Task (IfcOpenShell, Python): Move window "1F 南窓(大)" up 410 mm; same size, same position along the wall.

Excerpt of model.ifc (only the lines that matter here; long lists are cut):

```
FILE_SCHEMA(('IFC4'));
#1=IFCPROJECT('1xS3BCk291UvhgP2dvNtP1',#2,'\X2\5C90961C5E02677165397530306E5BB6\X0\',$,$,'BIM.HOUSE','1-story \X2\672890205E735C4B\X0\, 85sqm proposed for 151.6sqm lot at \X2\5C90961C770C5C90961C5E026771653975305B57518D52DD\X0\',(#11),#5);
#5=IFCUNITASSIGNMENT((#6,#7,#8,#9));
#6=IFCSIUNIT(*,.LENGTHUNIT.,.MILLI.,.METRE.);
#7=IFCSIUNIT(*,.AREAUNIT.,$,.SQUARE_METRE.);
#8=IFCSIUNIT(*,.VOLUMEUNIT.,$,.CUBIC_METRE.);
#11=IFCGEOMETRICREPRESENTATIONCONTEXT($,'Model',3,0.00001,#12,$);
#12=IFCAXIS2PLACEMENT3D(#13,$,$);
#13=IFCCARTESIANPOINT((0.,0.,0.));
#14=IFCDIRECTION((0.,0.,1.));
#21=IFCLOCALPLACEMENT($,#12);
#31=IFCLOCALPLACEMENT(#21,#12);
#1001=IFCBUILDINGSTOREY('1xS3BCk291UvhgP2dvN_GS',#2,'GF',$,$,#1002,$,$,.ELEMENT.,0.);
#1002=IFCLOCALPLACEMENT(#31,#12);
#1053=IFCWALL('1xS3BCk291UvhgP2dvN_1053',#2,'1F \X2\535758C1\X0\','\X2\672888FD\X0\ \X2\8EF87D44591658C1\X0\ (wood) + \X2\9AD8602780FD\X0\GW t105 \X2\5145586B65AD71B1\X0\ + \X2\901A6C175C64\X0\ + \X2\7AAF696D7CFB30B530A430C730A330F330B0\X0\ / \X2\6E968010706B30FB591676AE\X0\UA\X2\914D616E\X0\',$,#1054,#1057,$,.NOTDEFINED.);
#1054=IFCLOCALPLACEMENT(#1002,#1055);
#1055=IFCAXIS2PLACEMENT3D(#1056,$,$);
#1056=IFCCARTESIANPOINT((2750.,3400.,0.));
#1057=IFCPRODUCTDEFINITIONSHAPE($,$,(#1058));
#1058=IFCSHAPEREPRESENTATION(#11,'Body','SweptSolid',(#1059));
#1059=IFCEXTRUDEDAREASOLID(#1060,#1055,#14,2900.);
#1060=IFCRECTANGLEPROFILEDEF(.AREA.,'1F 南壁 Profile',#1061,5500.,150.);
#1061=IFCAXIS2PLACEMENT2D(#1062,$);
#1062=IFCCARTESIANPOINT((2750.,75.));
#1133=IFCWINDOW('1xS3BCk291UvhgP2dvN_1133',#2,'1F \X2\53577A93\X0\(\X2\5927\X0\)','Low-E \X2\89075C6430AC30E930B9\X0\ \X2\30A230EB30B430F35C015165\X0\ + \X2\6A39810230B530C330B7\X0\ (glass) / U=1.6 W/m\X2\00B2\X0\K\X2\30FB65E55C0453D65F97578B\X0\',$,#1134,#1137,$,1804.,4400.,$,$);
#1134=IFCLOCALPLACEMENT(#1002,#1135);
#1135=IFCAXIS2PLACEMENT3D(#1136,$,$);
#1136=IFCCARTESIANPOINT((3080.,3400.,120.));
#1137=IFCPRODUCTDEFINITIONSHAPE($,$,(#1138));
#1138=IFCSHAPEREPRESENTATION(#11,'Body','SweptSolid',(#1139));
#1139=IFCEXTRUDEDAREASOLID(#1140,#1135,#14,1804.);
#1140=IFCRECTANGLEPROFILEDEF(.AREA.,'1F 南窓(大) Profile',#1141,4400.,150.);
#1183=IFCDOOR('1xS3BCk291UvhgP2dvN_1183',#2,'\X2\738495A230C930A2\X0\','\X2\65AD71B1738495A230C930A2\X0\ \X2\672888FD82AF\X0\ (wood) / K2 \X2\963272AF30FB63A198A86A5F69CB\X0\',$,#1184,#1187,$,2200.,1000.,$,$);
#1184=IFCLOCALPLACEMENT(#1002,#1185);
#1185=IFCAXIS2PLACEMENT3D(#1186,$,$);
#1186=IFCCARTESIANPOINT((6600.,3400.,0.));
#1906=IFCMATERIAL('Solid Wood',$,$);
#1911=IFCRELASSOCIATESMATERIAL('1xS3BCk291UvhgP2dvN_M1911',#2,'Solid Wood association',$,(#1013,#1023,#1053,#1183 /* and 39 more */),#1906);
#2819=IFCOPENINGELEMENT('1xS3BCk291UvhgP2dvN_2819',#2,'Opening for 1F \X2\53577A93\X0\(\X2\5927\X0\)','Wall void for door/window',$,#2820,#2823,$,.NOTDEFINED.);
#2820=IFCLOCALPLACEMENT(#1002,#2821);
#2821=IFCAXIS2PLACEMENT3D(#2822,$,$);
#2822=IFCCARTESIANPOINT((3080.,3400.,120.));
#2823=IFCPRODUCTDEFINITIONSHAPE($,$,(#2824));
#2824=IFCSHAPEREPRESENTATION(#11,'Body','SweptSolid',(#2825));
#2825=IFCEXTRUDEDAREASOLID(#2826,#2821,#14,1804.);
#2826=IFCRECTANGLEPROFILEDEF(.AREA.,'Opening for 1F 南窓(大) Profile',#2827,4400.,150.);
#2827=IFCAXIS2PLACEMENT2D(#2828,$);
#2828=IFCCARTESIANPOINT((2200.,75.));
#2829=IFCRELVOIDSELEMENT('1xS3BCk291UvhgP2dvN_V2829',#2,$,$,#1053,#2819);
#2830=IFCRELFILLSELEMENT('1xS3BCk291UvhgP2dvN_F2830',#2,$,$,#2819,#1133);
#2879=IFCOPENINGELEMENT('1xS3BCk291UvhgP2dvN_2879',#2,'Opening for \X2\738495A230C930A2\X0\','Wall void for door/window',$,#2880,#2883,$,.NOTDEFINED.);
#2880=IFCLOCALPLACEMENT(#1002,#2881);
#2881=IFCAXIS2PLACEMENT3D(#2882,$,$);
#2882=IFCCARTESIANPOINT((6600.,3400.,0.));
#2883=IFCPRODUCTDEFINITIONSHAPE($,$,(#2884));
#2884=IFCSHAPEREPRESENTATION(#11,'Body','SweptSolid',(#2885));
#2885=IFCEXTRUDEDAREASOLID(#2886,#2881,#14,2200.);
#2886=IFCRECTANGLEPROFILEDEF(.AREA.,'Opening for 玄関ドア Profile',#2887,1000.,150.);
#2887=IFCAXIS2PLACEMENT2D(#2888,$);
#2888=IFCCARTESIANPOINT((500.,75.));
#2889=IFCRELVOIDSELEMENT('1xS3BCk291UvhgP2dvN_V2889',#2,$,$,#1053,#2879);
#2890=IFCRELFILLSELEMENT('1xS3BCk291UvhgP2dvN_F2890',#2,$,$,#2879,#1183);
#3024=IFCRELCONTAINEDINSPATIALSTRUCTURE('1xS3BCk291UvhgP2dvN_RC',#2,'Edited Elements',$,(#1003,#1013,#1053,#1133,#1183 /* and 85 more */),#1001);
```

```python
import numpy as np
import ifcopenshell
import ifcopenshell.api.geometry
import ifcopenshell.util.placement
import ifcopenshell.util.unit

model = ifcopenshell.open("model.ifc")
unit_scale = ifcopenshell.util.unit.calculate_unit_scale(model)

window = model.by_guid("1xS3BCk291UvhgP2dvN_1133")
opening = window.FillsVoids[0].RelatingOpeningElement
dz = 0.41 / unit_scale

shift = np.array([0.0, 0.0, dz])
# The window is not placed relative to its opening, so move both.
for product in (opening, window):
    matrix = ifcopenshell.util.placement.get_local_placement(product.ObjectPlacement)
    matrix[:3, 3] += shift
    ifcopenshell.api.geometry.edit_object_placement(model, product=product, matrix=matrix, is_si=False)

print(f"moved by {dz * unit_scale:+.3f} m")

model.write("model_edited.ifc")
```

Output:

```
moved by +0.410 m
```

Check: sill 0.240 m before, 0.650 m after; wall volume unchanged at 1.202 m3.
